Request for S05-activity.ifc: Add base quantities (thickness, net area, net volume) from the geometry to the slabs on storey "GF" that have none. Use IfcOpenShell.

First a look at what the model holds.

```python
import ifcopenshell
import ifcopenshell.util.element
import ifcopenshell.util.unit

model = ifcopenshell.open("S05-activity.ifc")
print(model.schema)
for unit_type in ("LENGTHUNIT", "AREAUNIT", "VOLUMEUNIT"):
    print(unit_type, ifcopenshell.util.unit.calculate_unit_scale(model, unit_type))
storey = next(s for s in model.by_type("IfcBuildingStorey") if s.Name == "GF")
slabs = [e for e in ifcopenshell.util.element.get_decomposition(storey) if e.is_a("IfcSlab")]
for e in sorted(slabs, key=lambda e: e.id()):
    print(e.id(), e.is_a(), e.Name, list(ifcopenshell.util.element.get_psets(e, qtos_only=True)), sep=" | ")
```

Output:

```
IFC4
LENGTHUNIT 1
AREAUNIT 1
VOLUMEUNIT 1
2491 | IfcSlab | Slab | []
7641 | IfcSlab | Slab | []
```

```python
import ifcopenshell
import ifcopenshell.api.pset
import ifcopenshell.geom
import ifcopenshell.util.element
import ifcopenshell.util.shape
import ifcopenshell.util.unit

model = ifcopenshell.open("S05-activity.ifc")
unit_scale = ifcopenshell.util.unit.calculate_unit_scale(model)
area_scale = ifcopenshell.util.unit.calculate_unit_scale(model, "AREAUNIT")
volume_scale = ifcopenshell.util.unit.calculate_unit_scale(model, "VOLUMEUNIT")
settings = ifcopenshell.geom.settings()

storey = next(s for s in model.by_type("IfcBuildingStorey") if s.Name == "GF")
slabs = [e for e in ifcopenshell.util.element.get_decomposition(storey) if e.is_a("IfcSlab")]

for e in sorted(slabs, key=lambda e: e.id()):
    if ifcopenshell.util.element.get_psets(e, qtos_only=True, should_inherit=False):
        continue
    # Geometry comes back in metres, in the element's own axes.
    shape = ifcopenshell.geom.create_shape(settings, e)
    values = {
        "Width": ifcopenshell.util.shape.get_z(shape.geometry) / unit_scale,
        "NetArea": ifcopenshell.util.shape.get_footprint_area(shape.geometry) / area_scale,
        "NetVolume": ifcopenshell.util.shape.get_volume(shape.geometry) / volume_scale,
    }
    qto = ifcopenshell.api.pset.add_qto(model, product=e, name="Qto_SlabBaseQuantities")
    ifcopenshell.api.pset.edit_qto(model, qto=qto, properties=values)
    print(e.id(), {k: round(v, 3) for k, v in values.items()})

model.write("S05-activity_v2.ifc")
```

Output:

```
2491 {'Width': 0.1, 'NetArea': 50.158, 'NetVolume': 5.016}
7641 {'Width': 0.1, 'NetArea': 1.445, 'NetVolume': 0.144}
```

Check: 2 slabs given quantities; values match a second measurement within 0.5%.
